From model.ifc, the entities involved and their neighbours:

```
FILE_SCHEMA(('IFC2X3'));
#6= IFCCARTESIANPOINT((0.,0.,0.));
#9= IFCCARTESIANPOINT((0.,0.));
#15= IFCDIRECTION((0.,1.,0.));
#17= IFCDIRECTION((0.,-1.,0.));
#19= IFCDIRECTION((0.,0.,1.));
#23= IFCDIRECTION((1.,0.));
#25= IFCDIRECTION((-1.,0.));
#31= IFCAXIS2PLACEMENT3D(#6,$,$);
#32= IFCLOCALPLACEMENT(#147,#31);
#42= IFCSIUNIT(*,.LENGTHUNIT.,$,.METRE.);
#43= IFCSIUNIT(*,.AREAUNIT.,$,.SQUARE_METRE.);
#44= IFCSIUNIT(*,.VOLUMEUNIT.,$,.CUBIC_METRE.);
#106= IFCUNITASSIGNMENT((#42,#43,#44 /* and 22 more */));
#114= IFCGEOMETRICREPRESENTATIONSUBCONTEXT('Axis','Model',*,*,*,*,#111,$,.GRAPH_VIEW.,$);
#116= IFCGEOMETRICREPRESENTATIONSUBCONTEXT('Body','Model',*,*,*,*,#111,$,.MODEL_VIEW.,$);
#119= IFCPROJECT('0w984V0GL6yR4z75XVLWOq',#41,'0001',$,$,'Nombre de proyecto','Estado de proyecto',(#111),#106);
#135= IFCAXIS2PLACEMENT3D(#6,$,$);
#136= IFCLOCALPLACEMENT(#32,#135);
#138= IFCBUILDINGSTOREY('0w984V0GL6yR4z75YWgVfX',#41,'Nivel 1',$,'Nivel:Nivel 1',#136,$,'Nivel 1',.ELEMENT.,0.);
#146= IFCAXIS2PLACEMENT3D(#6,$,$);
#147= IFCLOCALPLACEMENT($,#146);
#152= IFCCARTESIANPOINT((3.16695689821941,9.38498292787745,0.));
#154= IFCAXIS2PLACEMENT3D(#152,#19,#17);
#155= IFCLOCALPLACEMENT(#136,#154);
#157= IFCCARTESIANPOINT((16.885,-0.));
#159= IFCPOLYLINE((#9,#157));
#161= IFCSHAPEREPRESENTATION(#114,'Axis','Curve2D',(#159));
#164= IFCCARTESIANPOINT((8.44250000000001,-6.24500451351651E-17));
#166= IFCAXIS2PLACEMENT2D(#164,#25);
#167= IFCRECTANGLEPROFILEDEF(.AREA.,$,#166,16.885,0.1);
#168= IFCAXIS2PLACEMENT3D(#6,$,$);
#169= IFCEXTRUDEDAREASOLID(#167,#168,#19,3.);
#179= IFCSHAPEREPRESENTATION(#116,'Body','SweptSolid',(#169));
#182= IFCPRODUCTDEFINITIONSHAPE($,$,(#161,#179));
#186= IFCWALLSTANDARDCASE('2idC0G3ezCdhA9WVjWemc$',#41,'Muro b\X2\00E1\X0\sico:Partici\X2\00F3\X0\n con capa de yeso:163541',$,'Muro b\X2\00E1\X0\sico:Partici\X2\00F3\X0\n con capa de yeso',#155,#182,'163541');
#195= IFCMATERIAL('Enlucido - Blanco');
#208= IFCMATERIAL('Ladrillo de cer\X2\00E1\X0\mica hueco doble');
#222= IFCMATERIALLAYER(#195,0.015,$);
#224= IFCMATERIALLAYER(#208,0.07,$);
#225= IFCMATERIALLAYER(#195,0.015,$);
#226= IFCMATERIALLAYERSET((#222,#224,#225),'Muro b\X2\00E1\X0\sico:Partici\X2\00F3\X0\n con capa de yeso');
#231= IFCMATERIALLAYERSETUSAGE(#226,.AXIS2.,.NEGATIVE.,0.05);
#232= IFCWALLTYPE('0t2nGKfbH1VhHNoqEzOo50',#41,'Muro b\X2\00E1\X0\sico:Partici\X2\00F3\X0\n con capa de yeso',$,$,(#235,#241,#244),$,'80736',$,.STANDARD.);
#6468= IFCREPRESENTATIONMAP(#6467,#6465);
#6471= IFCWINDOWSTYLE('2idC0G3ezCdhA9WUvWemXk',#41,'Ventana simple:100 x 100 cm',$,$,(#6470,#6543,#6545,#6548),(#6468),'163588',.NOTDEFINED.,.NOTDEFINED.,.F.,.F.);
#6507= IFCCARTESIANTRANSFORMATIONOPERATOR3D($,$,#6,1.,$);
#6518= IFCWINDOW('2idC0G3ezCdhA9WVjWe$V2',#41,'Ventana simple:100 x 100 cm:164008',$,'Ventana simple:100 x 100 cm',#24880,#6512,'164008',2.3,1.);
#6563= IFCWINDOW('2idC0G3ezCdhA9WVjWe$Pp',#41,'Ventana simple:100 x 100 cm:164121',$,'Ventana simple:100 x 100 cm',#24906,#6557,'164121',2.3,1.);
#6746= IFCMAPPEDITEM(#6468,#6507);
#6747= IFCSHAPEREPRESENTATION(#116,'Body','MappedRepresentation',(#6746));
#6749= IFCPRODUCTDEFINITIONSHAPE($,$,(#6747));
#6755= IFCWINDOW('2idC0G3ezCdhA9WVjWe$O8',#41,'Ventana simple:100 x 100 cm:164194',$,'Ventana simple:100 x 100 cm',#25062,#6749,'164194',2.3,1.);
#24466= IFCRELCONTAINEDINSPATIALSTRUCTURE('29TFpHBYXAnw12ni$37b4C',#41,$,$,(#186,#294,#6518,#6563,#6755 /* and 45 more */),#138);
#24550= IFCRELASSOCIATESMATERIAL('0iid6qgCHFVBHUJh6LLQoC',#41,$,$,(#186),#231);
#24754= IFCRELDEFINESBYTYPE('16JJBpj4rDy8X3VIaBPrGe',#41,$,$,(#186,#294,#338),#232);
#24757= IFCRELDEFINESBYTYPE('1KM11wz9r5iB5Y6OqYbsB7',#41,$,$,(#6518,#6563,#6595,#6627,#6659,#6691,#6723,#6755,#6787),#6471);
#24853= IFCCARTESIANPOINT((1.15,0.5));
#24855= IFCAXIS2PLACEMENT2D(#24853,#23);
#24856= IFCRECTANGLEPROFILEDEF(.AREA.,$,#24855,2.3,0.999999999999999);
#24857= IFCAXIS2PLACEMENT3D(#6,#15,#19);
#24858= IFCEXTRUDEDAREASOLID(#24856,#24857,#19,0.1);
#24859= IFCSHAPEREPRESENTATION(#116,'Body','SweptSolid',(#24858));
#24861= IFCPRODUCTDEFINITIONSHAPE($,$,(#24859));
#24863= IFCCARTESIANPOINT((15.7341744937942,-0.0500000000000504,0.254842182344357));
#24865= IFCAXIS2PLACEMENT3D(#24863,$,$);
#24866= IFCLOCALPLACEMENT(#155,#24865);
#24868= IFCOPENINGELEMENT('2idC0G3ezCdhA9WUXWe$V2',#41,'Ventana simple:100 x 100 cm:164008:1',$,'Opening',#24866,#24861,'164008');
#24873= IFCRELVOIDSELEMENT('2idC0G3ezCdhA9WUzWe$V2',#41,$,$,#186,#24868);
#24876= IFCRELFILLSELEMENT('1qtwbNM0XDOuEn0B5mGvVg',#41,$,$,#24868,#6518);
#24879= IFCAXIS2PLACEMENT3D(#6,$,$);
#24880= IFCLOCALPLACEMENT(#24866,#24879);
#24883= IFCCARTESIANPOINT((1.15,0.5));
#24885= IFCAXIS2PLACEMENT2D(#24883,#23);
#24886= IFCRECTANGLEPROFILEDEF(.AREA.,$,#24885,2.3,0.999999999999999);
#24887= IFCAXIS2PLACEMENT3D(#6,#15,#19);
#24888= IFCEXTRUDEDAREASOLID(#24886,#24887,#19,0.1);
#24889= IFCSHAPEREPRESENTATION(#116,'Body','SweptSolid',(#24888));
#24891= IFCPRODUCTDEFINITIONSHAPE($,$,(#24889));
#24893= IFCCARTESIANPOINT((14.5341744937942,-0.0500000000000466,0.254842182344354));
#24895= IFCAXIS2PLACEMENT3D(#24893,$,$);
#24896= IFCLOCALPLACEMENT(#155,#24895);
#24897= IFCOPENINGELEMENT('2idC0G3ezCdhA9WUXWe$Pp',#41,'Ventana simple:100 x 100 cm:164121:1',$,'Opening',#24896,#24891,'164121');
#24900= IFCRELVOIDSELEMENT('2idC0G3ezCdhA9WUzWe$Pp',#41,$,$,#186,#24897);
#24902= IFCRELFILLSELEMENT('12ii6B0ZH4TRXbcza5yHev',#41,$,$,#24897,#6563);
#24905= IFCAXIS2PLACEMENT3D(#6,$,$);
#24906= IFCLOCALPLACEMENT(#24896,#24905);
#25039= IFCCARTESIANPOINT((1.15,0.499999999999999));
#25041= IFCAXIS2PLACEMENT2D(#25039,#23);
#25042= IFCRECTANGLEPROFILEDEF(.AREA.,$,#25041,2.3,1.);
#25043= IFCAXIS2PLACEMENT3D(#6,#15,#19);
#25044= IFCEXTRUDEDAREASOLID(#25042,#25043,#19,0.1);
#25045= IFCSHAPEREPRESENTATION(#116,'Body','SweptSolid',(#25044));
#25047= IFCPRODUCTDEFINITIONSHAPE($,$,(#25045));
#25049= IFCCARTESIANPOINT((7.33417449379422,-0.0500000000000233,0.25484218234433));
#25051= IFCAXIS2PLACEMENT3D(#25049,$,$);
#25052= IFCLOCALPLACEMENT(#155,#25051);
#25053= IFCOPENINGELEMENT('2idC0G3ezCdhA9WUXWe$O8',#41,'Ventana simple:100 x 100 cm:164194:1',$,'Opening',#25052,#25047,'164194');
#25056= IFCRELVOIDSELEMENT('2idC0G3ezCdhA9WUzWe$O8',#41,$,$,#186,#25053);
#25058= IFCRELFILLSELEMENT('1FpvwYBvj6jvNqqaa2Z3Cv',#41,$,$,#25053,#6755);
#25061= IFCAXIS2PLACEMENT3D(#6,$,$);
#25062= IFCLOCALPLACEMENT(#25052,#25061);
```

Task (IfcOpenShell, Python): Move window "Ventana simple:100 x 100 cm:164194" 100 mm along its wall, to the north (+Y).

```python
import ifcopenshell
import ifcopenshell.api.geometry
import ifcopenshell.util.placement

model = ifcopenshell.open("model.ifc")

window = model.by_guid("2idC0G3ezCdhA9WVjWe$O8")
opening = window.FillsVoids[0].RelatingOpeningElement
wall = opening.VoidsElements[0].RelatingBuildingElement

wall_matrix = ifcopenshell.util.placement.get_local_placement(wall.ObjectPlacement)
shift = wall_matrix[:3, 0] * -0.1
before = ifcopenshell.util.placement.get_local_placement(window.ObjectPlacement)[:3, 3].copy()

# The window is placed relative to its opening, so it follows when the opening moves.
matrix = ifcopenshell.util.placement.get_local_placement(opening.ObjectPlacement)
matrix[:3, 3] += shift
ifcopenshell.api.geometry.edit_object_placement(
    model, product=opening, matrix=matrix, is_si=False, should_transform_children=True
)

after = ifcopenshell.util.placement.get_local_placement(window.ObjectPlacement)[:3, 3]
print("window moved by", (after - before).round(3) + 0.0)

model.write("model_v2.ifc")
```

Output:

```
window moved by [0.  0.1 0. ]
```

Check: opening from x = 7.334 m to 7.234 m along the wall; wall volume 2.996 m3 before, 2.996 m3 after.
